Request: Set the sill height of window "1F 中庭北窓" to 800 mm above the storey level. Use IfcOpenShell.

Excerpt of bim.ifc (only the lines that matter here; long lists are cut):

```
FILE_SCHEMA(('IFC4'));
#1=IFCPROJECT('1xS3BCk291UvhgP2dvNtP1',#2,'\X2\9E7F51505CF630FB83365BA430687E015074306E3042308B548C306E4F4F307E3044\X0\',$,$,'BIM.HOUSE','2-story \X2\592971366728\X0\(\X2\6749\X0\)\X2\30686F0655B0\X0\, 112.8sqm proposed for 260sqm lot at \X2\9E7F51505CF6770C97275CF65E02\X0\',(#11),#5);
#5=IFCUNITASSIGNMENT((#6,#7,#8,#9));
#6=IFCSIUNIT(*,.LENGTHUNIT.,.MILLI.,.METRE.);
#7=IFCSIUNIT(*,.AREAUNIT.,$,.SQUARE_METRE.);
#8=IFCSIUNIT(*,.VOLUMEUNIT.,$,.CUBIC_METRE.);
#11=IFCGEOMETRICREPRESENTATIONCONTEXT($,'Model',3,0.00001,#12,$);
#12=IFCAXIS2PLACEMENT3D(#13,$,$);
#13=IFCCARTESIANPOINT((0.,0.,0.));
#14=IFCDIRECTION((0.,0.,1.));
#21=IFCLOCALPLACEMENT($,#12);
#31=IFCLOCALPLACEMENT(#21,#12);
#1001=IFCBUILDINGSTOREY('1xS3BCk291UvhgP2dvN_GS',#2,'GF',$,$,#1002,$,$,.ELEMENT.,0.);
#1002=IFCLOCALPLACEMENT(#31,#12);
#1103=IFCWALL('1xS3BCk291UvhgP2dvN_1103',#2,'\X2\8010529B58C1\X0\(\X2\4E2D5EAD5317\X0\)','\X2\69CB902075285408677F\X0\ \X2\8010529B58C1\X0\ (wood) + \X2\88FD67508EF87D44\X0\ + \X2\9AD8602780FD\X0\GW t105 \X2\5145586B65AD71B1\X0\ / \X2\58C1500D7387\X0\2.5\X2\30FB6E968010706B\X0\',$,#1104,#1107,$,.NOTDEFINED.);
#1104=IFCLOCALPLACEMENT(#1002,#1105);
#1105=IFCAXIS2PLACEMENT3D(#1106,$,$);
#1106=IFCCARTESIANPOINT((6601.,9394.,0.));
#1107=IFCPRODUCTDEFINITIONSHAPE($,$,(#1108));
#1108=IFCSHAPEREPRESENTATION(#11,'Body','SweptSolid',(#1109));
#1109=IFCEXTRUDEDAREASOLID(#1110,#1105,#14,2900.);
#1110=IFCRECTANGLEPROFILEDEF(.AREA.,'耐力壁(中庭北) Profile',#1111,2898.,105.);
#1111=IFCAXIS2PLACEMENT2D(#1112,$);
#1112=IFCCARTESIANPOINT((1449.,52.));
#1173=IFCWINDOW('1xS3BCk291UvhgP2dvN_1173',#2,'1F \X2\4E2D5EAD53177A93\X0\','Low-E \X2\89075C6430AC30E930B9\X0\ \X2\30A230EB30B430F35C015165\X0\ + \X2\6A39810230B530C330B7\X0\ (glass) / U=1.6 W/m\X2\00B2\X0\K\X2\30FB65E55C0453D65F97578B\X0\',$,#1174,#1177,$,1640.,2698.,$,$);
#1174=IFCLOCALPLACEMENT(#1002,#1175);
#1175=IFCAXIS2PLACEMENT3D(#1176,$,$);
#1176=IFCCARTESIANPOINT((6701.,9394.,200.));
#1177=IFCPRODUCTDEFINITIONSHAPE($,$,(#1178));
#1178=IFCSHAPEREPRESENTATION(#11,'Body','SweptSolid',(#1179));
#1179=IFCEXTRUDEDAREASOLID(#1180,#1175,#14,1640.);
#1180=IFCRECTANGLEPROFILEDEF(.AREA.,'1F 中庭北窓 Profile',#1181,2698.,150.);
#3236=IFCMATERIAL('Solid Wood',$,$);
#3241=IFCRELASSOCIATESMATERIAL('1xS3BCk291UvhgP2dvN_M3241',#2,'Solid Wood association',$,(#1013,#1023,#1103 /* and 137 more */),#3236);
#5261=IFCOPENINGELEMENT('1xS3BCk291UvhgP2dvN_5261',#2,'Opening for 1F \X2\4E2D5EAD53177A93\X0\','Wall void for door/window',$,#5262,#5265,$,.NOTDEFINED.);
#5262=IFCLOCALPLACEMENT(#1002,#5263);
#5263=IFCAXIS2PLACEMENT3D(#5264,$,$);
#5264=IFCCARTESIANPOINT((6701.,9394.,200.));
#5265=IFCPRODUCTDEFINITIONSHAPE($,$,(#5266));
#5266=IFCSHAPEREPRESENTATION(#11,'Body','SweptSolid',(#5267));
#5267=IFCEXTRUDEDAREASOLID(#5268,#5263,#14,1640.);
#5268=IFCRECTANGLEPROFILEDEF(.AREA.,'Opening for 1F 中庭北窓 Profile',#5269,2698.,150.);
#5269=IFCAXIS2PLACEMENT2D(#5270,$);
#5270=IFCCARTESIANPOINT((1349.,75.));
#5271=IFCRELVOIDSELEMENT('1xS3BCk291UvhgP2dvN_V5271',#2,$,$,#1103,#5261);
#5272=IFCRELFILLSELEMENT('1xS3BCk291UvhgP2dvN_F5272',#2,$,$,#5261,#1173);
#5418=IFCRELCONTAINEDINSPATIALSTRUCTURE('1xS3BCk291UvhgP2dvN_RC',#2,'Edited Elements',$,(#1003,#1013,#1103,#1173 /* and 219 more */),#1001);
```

```python
import numpy as np
import ifcopenshell
import ifcopenshell.api.geometry
import ifcopenshell.geom
import ifcopenshell.util.element
import ifcopenshell.util.placement
import ifcopenshell.util.shape
import ifcopenshell.util.unit

model = ifcopenshell.open("bim.ifc")
unit_scale = ifcopenshell.util.unit.calculate_unit_scale(model)

window = model.by_guid("1xS3BCk291UvhgP2dvN_1173")
opening = window.FillsVoids[0].RelatingOpeningElement
storey = ifcopenshell.util.element.get_container(window, ifc_class="IfcBuildingStorey")
level = ifcopenshell.util.placement.get_local_placement(storey.ObjectPlacement)[2, 3]

# The opening's origin need not be at the sill, so measure its lowest point.
shape = ifcopenshell.geom.create_shape(ifcopenshell.geom.settings(), opening)
bottom = ifcopenshell.util.shape.get_shape_bottom_elevation(shape, shape.geometry) / unit_scale
dz = level + 0.8 / unit_scale - bottom

shift = np.array([0.0, 0.0, dz])
# The window is not placed relative to its opening, so move both.
for product in (opening, window):
    matrix = ifcopenshell.util.placement.get_local_placement(product.ObjectPlacement)
    matrix[:3, 3] += shift
    ifcopenshell.api.geometry.edit_object_placement(model, product=product, matrix=matrix, is_si=False)

print(f"moved by {dz * unit_scale:+.3f} m")

model.write("bim_rev.ifc")
```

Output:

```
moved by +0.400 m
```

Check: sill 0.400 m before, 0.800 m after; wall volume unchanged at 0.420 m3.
